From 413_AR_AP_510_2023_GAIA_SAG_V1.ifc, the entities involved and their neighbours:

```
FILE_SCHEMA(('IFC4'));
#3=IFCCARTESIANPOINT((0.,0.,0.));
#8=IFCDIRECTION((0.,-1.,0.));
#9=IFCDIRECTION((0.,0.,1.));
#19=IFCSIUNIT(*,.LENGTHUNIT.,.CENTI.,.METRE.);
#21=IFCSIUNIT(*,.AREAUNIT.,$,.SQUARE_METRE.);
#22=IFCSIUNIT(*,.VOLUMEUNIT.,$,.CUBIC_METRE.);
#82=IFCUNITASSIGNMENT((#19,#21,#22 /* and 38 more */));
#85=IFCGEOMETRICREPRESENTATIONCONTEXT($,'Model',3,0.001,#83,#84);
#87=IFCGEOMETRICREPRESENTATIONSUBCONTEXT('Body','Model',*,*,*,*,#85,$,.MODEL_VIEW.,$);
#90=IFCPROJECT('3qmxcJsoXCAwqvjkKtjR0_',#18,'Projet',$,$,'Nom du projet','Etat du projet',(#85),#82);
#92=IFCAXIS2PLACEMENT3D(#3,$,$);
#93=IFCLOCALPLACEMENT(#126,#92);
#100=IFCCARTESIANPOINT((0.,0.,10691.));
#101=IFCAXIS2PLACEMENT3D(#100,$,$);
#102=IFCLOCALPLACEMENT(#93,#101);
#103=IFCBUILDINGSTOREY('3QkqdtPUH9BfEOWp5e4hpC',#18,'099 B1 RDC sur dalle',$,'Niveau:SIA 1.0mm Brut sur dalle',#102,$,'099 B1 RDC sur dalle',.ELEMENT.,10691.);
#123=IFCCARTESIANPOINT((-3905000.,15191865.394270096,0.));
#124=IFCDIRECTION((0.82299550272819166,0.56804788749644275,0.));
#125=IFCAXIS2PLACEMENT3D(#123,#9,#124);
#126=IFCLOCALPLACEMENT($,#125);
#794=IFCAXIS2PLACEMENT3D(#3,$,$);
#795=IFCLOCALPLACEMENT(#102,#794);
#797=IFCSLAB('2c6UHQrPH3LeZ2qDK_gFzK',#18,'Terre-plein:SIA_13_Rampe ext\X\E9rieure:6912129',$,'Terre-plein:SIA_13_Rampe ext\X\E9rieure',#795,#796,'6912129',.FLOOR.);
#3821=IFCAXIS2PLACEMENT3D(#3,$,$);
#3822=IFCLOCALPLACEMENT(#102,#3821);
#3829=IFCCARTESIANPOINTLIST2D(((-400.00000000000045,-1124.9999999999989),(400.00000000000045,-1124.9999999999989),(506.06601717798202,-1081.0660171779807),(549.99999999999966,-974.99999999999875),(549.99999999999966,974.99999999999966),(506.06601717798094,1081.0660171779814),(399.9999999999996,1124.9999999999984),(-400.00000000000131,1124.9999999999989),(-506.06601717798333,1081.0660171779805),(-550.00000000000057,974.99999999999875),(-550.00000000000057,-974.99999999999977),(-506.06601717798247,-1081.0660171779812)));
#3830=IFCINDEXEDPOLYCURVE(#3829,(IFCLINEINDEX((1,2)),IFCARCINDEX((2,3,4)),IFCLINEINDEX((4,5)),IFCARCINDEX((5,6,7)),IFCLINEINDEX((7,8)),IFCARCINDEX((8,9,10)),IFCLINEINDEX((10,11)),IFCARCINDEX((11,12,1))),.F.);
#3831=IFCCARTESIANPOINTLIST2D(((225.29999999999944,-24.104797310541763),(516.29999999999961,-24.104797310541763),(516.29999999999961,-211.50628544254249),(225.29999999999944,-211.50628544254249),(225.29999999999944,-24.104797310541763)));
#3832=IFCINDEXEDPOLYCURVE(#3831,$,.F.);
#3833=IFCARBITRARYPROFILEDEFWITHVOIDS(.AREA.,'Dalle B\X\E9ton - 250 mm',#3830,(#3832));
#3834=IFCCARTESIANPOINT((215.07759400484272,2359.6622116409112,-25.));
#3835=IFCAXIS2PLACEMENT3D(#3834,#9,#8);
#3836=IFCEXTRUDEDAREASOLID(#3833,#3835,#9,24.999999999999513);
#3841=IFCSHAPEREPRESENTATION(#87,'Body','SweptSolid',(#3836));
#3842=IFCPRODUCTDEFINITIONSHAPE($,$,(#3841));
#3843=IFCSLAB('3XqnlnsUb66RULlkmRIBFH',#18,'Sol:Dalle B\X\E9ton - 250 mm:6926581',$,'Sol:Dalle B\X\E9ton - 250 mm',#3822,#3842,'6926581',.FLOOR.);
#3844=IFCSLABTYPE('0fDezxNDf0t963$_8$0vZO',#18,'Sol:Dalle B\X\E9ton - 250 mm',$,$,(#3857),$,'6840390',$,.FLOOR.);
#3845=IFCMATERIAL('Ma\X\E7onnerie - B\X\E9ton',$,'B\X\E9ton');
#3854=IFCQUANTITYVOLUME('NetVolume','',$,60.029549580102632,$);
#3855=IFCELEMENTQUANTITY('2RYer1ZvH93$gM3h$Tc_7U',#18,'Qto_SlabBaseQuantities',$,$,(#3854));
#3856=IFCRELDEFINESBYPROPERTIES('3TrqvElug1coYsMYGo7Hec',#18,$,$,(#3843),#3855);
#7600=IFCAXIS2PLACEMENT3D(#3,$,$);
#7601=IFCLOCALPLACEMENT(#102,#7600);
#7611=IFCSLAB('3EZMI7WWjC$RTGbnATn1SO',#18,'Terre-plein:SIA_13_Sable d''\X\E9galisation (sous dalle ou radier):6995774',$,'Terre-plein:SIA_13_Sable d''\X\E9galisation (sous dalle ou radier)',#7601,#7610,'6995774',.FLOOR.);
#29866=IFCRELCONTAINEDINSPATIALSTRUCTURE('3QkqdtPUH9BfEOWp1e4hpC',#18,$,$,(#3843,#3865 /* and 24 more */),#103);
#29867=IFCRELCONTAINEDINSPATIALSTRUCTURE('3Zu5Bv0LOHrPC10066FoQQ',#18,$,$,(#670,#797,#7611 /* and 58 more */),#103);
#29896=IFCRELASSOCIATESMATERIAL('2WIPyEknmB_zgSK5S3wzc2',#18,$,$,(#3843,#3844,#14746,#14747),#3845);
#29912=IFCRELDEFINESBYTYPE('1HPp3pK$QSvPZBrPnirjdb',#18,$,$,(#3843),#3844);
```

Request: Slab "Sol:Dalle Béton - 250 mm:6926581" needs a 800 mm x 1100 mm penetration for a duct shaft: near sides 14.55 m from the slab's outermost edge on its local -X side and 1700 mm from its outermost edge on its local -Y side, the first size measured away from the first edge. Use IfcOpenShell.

```python
import numpy as np
import ifcopenshell
import ifcopenshell.api.feature
import ifcopenshell.api.geometry
import ifcopenshell.api.pset
import ifcopenshell.api.root
import ifcopenshell.geom
import ifcopenshell.util.element
import ifcopenshell.util.placement
import ifcopenshell.util.representation
import ifcopenshell.util.shape
import ifcopenshell.util.unit

model = ifcopenshell.open("413_AR_AP_510_2023_GAIA_SAG_V1.ifc")
unit_scale = ifcopenshell.util.unit.calculate_unit_scale(model)
volume_scale = ifcopenshell.util.unit.calculate_unit_scale(model, "VOLUMEUNIT")
settings = ifcopenshell.geom.settings()


def volume(element):
    """Net volume in cubic metres, openings subtracted."""
    shape = ifcopenshell.geom.create_shape(settings, element)
    return ifcopenshell.util.shape.get_volume(shape.geometry)


slab = model.by_guid("3XqnlnsUb66RULlkmRIBFH")
before = volume(slab)

# Extent in the slab's own axes, in metres. The edges named are its -X and -Y sides.
slab_shape = ifcopenshell.geom.create_shape(settings, slab)
vertices = ifcopenshell.util.shape.get_vertices(slab_shape.geometry)
x_min, y_min, bottom = vertices.min(axis=0)
top = vertices[:, 2].max()

opening = ifcopenshell.api.root.create_entity(model, ifc_class="IfcOpeningElement", name="Duct shaft opening", predefined_type="OPENING")
context = ifcopenshell.util.representation.get_context(model, "Model", "Body", "MODEL_VIEW")
width, depth = 0.8, 1.1
outline = [(0.0, 0.0), (width, 0.0), (width, depth), (0.0, depth), (0.0, 0.0)]
# Overshoot both faces by 50 mm so the cut is clean.
shape = ifcopenshell.api.geometry.add_slab_representation(
    model, context=context, depth=top - bottom + 0.1, polyline=outline
)
ifcopenshell.api.geometry.assign_representation(model, product=opening, representation=shape)

matrix = ifcopenshell.util.placement.get_local_placement(slab.ObjectPlacement)
matrix[:, 3] = matrix @ np.append(np.array([x_min + 14.55, y_min + 1.7, bottom - 0.05]) / unit_scale, 1.0)
ifcopenshell.api.geometry.edit_object_placement(model, product=opening, matrix=matrix, is_si=False)
ifcopenshell.api.feature.add_feature(model, feature=opening, element=slab)

after = volume(slab)

# Update the slab's stored quantities.
qto = model.by_id(ifcopenshell.util.element.get_pset(slab, "Qto_SlabBaseQuantities", should_inherit=False)["id"])
ifcopenshell.api.pset.edit_qto(model, qto=qto, properties={"NetVolume": after / volume_scale})

print(f"slab volume {before:.3f} -> {after:.3f} m3")

model.write("413_AR_AP_510_2023_GAIA_SAG_V1_rev.ifc")
```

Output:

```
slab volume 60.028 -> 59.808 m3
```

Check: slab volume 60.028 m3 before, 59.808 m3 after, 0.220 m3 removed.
